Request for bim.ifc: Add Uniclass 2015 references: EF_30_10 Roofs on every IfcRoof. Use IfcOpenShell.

First a look at what the model holds.

```python
import ifcopenshell

model = ifcopenshell.open("bim.ifc")
print(model.schema)
print("classifications:", [c.Name for c in model.by_type("IfcClassification")])
for ifc_class in ("IfcDoor", "IfcRoof", "IfcStair", "IfcWall", "IfcWindow"):
    print(ifc_class, len(model.by_type(ifc_class)))
```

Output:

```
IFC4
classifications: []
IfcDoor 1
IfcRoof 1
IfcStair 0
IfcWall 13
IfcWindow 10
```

```python
import ifcopenshell
import ifcopenshell.api.classification

model = ifcopenshell.open("bim.ifc")

system = ifcopenshell.api.classification.add_classification(model, classification="Uniclass 2015")

codes = {
    "IfcRoof": ("EF_30_10", "Roofs"),
}
for ifc_class, (code, name) in codes.items():
    products = model.by_type(ifc_class)
    ifcopenshell.api.classification.add_reference(
        model, products=products, classification=system, identification=code, name=name
    )
    print(code, len(products))

model.write("bim-out.ifc")
```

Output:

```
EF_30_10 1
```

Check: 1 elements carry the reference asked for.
